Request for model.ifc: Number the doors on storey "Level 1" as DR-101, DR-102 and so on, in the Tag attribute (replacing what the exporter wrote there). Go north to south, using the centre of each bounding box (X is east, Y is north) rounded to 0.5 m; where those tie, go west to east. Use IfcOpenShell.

First a look at what the model holds.

```python
import ifcopenshell
import ifcopenshell.util.element
import ifcopenshell.util.placement

model = ifcopenshell.open("model.ifc")
print(model.schema)
storey = next(s for s in model.by_type("IfcBuildingStorey") if s.Name == "Level 1")
doors = [e for e in ifcopenshell.util.element.get_decomposition(storey) if e.is_a("IfcDoor")]
for e in sorted(doors, key=lambda e: e.id()):
    origin = ifcopenshell.util.placement.get_local_placement(e.ObjectPlacement)[:3, 3]
    print(e.id(), e.Tag, e.Name, origin.round(2) + 0.0, sep=" | ")
```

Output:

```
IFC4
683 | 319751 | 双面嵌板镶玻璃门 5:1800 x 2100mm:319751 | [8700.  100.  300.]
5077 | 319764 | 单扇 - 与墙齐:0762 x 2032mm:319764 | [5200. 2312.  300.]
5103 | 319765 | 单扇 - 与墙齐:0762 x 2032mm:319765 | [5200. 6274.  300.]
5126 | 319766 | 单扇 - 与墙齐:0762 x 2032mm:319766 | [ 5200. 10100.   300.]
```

```python
import ifcopenshell
import ifcopenshell.geom
import ifcopenshell.util.element
import ifcopenshell.util.shape

model = ifcopenshell.open("model.ifc")
settings = ifcopenshell.geom.settings()
settings.set("use-world-coords", True)


def centre(element):
    shape = ifcopenshell.geom.create_shape(settings, element)
    return ifcopenshell.util.shape.get_bbox_centroid(shape.geometry)


storey = next(s for s in model.by_type("IfcBuildingStorey") if s.Name == "Level 1")
doors = [e for e in ifcopenshell.util.element.get_decomposition(storey) if e.is_a("IfcDoor")]

# Insertion points can sit at a corner or the storey origin, so sort by the geometry (in metres).
centres = {e: centre(e) for e in doors}
doors.sort(key=lambda e: (-round(centres[e][1] / 0.5), centres[e][0]))

for i, e in enumerate(doors, start=1):
    number = f"DR-1{i:02d}"
    e.Tag = number
    print(e.id(), number)

model.write("model-out.ifc")
```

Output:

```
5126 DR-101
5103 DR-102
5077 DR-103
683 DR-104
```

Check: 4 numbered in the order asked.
